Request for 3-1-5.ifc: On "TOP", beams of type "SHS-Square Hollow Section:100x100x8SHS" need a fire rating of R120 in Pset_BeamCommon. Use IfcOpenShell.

First a look at what the model holds.

```python
import ifcopenshell
import ifcopenshell.util.element

model = ifcopenshell.open("3-1-5.ifc")
print(model.schema)
storey = next(s for s in model.by_type("IfcBuildingStorey") if s.Name == "TOP")
beams = [e for e in ifcopenshell.util.element.get_decomposition(storey) if e.is_a("IfcBeam")]
seen = {}
for e in beams:
    element_type = ifcopenshell.util.element.get_type(e)
    key = (element_type.Name if element_type != e and element_type else None, ifcopenshell.util.element.get_pset(e, "Pset_BeamCommon", "FireRating"))
    seen[key] = seen.get(key, 0) + 1
for (name, value), count in sorted(seen.items(), key=str):
    print(count, "x", name, "|", value)
```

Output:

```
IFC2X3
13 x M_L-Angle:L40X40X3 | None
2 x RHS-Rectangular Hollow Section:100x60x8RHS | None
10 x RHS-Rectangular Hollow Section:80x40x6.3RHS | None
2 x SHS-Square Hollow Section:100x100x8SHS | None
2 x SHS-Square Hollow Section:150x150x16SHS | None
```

```python
import ifcopenshell
import ifcopenshell.api.pset
import ifcopenshell.util.element

model = ifcopenshell.open("3-1-5.ifc")

storey = next(s for s in model.by_type("IfcBuildingStorey") if s.Name == "TOP")
beams = [e for e in ifcopenshell.util.element.get_decomposition(storey) if e.is_a("IfcBeam")]

count = 0
for e in beams:
    element_type = ifcopenshell.util.element.get_type(e)
    if element_type in (None, e) or element_type.Name != "SHS-Square Hollow Section:100x100x8SHS":
        continue
    # add_pset returns the element's existing set when there is one.
    pset = ifcopenshell.api.pset.add_pset(model, product=e, name="Pset_BeamCommon")
    ifcopenshell.api.pset.edit_pset(model, pset=pset, properties={"FireRating": "R120"})
    count += 1

print(count, "beams updated")

model.write("3-1-5_v2.ifc")
```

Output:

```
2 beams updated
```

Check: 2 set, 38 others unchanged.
